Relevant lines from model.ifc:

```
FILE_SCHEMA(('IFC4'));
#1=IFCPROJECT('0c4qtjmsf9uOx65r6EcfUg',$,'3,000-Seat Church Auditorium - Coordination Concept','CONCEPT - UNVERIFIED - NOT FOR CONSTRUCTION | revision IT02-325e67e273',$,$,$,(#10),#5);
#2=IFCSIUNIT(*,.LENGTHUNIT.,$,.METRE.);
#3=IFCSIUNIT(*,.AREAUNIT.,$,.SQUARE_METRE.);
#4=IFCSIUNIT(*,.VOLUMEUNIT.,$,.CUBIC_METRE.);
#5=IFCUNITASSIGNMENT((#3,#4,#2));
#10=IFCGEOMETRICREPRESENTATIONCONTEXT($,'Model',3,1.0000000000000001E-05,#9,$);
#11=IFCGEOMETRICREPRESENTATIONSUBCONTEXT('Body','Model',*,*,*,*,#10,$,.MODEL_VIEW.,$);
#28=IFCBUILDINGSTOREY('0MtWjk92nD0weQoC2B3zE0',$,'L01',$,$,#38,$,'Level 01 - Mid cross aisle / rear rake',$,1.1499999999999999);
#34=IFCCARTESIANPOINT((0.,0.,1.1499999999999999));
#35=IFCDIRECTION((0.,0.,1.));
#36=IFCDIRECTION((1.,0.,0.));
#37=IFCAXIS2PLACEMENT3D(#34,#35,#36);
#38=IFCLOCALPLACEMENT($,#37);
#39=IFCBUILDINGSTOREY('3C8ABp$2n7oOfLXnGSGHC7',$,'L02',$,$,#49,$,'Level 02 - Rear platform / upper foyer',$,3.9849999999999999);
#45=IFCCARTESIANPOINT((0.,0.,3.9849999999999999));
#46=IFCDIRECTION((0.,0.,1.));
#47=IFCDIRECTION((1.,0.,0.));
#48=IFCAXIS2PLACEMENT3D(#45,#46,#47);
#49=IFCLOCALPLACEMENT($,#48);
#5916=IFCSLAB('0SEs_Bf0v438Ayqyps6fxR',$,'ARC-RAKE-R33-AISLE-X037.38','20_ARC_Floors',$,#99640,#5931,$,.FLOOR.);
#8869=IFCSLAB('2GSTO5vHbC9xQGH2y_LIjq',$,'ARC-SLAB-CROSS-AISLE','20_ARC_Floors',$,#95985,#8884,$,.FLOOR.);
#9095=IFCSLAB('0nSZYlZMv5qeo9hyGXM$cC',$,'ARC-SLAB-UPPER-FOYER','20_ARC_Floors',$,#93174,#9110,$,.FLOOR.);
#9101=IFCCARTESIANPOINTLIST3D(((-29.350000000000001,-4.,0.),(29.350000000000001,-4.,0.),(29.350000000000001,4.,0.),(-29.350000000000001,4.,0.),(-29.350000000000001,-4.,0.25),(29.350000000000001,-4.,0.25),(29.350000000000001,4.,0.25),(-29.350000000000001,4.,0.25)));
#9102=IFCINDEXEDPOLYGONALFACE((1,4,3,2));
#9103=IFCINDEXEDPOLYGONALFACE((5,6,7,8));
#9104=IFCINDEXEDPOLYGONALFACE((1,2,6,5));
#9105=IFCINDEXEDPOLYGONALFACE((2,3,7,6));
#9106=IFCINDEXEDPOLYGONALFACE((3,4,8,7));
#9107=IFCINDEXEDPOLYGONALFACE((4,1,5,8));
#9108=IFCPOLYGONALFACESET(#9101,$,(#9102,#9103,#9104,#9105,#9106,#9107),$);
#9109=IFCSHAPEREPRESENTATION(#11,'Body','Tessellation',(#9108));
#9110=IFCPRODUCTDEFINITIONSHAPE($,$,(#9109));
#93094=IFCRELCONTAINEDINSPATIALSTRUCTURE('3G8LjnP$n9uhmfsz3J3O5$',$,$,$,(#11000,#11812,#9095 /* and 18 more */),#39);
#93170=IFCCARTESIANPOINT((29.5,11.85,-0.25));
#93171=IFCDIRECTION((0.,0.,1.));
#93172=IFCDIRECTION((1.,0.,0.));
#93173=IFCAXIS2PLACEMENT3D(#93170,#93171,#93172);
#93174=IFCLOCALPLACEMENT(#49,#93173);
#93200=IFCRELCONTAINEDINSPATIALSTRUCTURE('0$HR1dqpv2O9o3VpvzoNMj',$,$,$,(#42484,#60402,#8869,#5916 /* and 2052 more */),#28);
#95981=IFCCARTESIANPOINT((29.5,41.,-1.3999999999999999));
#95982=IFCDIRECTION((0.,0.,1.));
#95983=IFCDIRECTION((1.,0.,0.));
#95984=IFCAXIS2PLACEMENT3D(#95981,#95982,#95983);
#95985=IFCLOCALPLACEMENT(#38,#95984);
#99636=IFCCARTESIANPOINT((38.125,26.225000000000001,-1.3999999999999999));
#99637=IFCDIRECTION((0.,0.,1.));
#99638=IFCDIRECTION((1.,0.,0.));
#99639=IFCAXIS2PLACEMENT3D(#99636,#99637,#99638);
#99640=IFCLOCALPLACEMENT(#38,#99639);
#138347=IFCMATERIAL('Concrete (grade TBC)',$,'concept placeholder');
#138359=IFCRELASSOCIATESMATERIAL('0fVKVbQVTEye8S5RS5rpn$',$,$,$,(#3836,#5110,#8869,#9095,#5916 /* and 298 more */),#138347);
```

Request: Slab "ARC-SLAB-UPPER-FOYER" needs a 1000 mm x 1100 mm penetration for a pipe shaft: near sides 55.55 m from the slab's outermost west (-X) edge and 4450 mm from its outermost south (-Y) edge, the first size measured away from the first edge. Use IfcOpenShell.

```python
import numpy as np
import ifcopenshell
import ifcopenshell.api.feature
import ifcopenshell.api.geometry
import ifcopenshell.api.root
import ifcopenshell.geom
import ifcopenshell.util.placement
import ifcopenshell.util.representation
import ifcopenshell.util.shape
import ifcopenshell.util.unit

model = ifcopenshell.open("model.ifc")
unit_scale = ifcopenshell.util.unit.calculate_unit_scale(model)
settings = ifcopenshell.geom.settings()


def volume(element):
    """Net volume in cubic metres, openings subtracted."""
    shape = ifcopenshell.geom.create_shape(settings, element)
    return ifcopenshell.util.shape.get_volume(shape.geometry)


slab = model.by_guid("0nSZYlZMv5qeo9hyGXM$cC")
before = volume(slab)

# Extent in the slab's own axes, in metres. The edges named are its -X and -Y sides.
slab_shape = ifcopenshell.geom.create_shape(settings, slab)
vertices = ifcopenshell.util.shape.get_vertices(slab_shape.geometry)
x_min, y_min, bottom = vertices.min(axis=0)
top = vertices[:, 2].max()

opening = ifcopenshell.api.root.create_entity(model, ifc_class="IfcOpeningElement", name="Pipe shaft opening", predefined_type="OPENING")
context = ifcopenshell.util.representation.get_context(model, "Model", "Body", "MODEL_VIEW")
width, depth = 1, 1.1
outline = [(0.0, 0.0), (width, 0.0), (width, depth), (0.0, depth), (0.0, 0.0)]
# Overshoot both faces by 50 mm so the cut is clean.
shape = ifcopenshell.api.geometry.add_slab_representation(
    model, context=context, depth=top - bottom + 0.1, polyline=outline
)
ifcopenshell.api.geometry.assign_representation(model, product=opening, representation=shape)

matrix = ifcopenshell.util.placement.get_local_placement(slab.ObjectPlacement)
matrix[:, 3] = matrix @ np.append(np.array([x_min + 55.55, y_min + 4.45, bottom - 0.05]) / unit_scale, 1.0)
ifcopenshell.api.geometry.edit_object_placement(model, product=opening, matrix=matrix, is_si=False)
ifcopenshell.api.feature.add_feature(model, feature=opening, element=slab)

after = volume(slab)

print(f"slab volume {before:.3f} -> {after:.3f} m3")

model.write("model-out.ifc")
```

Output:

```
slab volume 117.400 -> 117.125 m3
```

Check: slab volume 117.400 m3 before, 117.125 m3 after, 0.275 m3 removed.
